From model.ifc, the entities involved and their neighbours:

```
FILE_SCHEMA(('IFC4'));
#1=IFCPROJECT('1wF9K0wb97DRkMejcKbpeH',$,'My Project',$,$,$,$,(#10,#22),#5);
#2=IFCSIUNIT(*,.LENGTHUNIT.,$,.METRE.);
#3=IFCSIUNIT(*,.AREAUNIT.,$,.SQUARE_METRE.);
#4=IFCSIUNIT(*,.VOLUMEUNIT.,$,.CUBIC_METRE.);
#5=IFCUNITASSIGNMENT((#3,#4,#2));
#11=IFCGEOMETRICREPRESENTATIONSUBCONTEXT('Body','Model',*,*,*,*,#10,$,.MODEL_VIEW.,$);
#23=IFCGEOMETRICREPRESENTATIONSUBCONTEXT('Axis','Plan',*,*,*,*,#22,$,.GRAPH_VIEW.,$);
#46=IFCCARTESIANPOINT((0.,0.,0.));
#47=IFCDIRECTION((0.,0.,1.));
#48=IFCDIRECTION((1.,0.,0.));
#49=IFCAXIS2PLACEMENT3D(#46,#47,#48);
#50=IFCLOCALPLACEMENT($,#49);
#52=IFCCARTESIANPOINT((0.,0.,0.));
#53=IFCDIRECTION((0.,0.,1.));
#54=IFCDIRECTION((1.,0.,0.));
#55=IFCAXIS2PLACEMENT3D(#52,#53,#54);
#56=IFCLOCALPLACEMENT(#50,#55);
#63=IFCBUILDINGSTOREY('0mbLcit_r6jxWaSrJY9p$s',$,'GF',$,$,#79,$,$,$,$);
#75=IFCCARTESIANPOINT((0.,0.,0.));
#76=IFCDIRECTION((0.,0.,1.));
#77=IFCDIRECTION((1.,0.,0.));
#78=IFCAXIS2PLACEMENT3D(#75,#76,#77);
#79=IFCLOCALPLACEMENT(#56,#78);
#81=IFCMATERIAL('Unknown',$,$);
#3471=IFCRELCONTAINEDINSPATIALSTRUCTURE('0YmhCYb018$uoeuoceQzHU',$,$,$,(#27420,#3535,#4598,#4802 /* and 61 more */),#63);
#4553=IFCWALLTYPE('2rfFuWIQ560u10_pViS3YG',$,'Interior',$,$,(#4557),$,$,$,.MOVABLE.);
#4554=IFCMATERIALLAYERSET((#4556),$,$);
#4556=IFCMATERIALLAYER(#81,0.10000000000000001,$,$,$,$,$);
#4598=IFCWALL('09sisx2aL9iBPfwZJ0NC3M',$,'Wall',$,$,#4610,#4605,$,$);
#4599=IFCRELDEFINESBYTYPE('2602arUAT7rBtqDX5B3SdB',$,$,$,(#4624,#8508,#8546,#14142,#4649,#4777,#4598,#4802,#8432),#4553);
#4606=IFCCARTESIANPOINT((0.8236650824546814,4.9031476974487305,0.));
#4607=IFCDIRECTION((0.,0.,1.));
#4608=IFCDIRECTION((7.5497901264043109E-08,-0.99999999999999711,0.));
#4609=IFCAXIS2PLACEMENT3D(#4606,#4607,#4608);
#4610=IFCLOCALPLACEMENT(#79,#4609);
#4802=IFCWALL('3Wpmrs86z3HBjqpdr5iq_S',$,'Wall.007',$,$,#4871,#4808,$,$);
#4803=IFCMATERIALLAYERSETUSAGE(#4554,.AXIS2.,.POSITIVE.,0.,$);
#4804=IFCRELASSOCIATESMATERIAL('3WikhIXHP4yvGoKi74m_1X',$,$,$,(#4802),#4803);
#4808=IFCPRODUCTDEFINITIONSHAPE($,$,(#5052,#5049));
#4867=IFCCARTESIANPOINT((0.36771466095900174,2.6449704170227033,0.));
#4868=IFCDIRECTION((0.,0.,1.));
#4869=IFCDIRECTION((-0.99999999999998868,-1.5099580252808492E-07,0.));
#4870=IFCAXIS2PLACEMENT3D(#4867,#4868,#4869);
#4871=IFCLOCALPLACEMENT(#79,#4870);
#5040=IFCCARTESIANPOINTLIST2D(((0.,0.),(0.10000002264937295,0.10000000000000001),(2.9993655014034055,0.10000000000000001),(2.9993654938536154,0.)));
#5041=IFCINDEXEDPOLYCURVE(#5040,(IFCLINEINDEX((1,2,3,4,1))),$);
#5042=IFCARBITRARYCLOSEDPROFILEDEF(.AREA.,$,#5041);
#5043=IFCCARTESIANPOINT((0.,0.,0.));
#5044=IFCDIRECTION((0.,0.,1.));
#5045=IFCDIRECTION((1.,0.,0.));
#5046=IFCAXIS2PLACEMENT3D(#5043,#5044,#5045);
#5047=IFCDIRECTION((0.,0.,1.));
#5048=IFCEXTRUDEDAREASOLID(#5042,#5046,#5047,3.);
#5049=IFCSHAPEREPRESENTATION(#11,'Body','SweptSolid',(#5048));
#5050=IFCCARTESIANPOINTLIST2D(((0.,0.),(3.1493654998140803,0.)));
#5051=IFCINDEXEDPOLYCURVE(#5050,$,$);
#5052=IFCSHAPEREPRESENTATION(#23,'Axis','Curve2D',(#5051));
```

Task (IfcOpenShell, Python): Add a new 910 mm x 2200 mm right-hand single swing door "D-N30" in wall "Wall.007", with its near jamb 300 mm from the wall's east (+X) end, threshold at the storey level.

```python
import numpy as np
import ifcopenshell
import ifcopenshell.api.feature
import ifcopenshell.api.geometry
import ifcopenshell.api.root
import ifcopenshell.api.spatial
import ifcopenshell.geom
import ifcopenshell.util.element
import ifcopenshell.util.placement
import ifcopenshell.util.representation
import ifcopenshell.util.shape
import ifcopenshell.util.unit

model = ifcopenshell.open("model.ifc")
unit_scale = ifcopenshell.util.unit.calculate_unit_scale(model)
settings = ifcopenshell.geom.settings()


def volume(element):
    """Net volume in cubic metres, openings subtracted."""
    shape = ifcopenshell.geom.create_shape(settings, element)
    return ifcopenshell.util.shape.get_volume(shape.geometry)


wall = model.by_id(4802)
storey = ifcopenshell.util.element.get_container(wall, ifc_class="IfcBuildingStorey")
context = ifcopenshell.util.representation.get_context(model, "Model", "Body", "MODEL_VIEW")
before = volume(wall)

width, height, from_end, sill = 0.91, 2.2, 0.3, 0.0  # metres

# The wall runs along its own X axis, and the end named is its -X end.
wall_shape = ifcopenshell.geom.create_shape(settings, wall)
x, y, z = ifcopenshell.util.shape.get_vertices(wall_shape.geometry).T
start = x.min() + from_end
face, thickness = float(y.min()), float(y.max() - y.min())
wall_matrix = ifcopenshell.util.placement.get_local_placement(wall.ObjectPlacement)
level = ifcopenshell.util.placement.get_local_placement(storey.ObjectPlacement)[2, 3]


def in_wall(x, y):
    """Placement at x, y metres in the wall's axes, at sill height."""
    matrix = wall_matrix.copy()
    matrix[:, 3] = wall_matrix @ np.array([x / unit_scale, y / unit_scale, 0.0, 1.0])
    matrix[2, 3] = level + sill / unit_scale
    return matrix


# Opening: a box that overshoots both wall faces by 50 mm.
opening = ifcopenshell.api.root.create_entity(model, ifc_class="IfcOpeningElement", predefined_type="OPENING")
box = ifcopenshell.api.geometry.add_wall_representation(
    model, context=context, length=width, height=height, thickness=thickness + 0.1
)
ifcopenshell.api.geometry.assign_representation(model, product=opening, representation=box)
ifcopenshell.api.geometry.edit_object_placement(model, product=opening, matrix=in_wall(start, face - 0.05), is_si=False)
ifcopenshell.api.feature.add_feature(model, feature=opening, element=wall)

door = ifcopenshell.api.root.create_entity(model, ifc_class="IfcDoor", name="D-N30", predefined_type="DOOR")
door.OverallWidth, door.OverallHeight = width / unit_scale, height / unit_scale
door.OperationType = "SINGLE_SWING_RIGHT"
body = ifcopenshell.api.geometry.add_door_representation(
    model,
    context=context,
    overall_width=door.OverallWidth,
    overall_height=door.OverallHeight,
    operation_type="SINGLE_SWING_RIGHT",
    lining_properties={"LiningDepth": thickness / unit_scale, "ThresholdDepth": thickness / unit_scale},
)
ifcopenshell.api.geometry.assign_representation(model, product=door, representation=body)
ifcopenshell.api.spatial.assign_container(model, products=[door], relating_structure=storey)
ifcopenshell.api.feature.add_filling(model, opening=opening, element=door)

# The lining spans the wall, so the door starts at the wall face.
ifcopenshell.api.geometry.edit_object_placement(model, product=door, matrix=in_wall(start, face), is_si=False)

after = volume(wall)

print(f"wall volume {before:.3f} -> {after:.3f} m3")

model.write("model_edited.ifc")
```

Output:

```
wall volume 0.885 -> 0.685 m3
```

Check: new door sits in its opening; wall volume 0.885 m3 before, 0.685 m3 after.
